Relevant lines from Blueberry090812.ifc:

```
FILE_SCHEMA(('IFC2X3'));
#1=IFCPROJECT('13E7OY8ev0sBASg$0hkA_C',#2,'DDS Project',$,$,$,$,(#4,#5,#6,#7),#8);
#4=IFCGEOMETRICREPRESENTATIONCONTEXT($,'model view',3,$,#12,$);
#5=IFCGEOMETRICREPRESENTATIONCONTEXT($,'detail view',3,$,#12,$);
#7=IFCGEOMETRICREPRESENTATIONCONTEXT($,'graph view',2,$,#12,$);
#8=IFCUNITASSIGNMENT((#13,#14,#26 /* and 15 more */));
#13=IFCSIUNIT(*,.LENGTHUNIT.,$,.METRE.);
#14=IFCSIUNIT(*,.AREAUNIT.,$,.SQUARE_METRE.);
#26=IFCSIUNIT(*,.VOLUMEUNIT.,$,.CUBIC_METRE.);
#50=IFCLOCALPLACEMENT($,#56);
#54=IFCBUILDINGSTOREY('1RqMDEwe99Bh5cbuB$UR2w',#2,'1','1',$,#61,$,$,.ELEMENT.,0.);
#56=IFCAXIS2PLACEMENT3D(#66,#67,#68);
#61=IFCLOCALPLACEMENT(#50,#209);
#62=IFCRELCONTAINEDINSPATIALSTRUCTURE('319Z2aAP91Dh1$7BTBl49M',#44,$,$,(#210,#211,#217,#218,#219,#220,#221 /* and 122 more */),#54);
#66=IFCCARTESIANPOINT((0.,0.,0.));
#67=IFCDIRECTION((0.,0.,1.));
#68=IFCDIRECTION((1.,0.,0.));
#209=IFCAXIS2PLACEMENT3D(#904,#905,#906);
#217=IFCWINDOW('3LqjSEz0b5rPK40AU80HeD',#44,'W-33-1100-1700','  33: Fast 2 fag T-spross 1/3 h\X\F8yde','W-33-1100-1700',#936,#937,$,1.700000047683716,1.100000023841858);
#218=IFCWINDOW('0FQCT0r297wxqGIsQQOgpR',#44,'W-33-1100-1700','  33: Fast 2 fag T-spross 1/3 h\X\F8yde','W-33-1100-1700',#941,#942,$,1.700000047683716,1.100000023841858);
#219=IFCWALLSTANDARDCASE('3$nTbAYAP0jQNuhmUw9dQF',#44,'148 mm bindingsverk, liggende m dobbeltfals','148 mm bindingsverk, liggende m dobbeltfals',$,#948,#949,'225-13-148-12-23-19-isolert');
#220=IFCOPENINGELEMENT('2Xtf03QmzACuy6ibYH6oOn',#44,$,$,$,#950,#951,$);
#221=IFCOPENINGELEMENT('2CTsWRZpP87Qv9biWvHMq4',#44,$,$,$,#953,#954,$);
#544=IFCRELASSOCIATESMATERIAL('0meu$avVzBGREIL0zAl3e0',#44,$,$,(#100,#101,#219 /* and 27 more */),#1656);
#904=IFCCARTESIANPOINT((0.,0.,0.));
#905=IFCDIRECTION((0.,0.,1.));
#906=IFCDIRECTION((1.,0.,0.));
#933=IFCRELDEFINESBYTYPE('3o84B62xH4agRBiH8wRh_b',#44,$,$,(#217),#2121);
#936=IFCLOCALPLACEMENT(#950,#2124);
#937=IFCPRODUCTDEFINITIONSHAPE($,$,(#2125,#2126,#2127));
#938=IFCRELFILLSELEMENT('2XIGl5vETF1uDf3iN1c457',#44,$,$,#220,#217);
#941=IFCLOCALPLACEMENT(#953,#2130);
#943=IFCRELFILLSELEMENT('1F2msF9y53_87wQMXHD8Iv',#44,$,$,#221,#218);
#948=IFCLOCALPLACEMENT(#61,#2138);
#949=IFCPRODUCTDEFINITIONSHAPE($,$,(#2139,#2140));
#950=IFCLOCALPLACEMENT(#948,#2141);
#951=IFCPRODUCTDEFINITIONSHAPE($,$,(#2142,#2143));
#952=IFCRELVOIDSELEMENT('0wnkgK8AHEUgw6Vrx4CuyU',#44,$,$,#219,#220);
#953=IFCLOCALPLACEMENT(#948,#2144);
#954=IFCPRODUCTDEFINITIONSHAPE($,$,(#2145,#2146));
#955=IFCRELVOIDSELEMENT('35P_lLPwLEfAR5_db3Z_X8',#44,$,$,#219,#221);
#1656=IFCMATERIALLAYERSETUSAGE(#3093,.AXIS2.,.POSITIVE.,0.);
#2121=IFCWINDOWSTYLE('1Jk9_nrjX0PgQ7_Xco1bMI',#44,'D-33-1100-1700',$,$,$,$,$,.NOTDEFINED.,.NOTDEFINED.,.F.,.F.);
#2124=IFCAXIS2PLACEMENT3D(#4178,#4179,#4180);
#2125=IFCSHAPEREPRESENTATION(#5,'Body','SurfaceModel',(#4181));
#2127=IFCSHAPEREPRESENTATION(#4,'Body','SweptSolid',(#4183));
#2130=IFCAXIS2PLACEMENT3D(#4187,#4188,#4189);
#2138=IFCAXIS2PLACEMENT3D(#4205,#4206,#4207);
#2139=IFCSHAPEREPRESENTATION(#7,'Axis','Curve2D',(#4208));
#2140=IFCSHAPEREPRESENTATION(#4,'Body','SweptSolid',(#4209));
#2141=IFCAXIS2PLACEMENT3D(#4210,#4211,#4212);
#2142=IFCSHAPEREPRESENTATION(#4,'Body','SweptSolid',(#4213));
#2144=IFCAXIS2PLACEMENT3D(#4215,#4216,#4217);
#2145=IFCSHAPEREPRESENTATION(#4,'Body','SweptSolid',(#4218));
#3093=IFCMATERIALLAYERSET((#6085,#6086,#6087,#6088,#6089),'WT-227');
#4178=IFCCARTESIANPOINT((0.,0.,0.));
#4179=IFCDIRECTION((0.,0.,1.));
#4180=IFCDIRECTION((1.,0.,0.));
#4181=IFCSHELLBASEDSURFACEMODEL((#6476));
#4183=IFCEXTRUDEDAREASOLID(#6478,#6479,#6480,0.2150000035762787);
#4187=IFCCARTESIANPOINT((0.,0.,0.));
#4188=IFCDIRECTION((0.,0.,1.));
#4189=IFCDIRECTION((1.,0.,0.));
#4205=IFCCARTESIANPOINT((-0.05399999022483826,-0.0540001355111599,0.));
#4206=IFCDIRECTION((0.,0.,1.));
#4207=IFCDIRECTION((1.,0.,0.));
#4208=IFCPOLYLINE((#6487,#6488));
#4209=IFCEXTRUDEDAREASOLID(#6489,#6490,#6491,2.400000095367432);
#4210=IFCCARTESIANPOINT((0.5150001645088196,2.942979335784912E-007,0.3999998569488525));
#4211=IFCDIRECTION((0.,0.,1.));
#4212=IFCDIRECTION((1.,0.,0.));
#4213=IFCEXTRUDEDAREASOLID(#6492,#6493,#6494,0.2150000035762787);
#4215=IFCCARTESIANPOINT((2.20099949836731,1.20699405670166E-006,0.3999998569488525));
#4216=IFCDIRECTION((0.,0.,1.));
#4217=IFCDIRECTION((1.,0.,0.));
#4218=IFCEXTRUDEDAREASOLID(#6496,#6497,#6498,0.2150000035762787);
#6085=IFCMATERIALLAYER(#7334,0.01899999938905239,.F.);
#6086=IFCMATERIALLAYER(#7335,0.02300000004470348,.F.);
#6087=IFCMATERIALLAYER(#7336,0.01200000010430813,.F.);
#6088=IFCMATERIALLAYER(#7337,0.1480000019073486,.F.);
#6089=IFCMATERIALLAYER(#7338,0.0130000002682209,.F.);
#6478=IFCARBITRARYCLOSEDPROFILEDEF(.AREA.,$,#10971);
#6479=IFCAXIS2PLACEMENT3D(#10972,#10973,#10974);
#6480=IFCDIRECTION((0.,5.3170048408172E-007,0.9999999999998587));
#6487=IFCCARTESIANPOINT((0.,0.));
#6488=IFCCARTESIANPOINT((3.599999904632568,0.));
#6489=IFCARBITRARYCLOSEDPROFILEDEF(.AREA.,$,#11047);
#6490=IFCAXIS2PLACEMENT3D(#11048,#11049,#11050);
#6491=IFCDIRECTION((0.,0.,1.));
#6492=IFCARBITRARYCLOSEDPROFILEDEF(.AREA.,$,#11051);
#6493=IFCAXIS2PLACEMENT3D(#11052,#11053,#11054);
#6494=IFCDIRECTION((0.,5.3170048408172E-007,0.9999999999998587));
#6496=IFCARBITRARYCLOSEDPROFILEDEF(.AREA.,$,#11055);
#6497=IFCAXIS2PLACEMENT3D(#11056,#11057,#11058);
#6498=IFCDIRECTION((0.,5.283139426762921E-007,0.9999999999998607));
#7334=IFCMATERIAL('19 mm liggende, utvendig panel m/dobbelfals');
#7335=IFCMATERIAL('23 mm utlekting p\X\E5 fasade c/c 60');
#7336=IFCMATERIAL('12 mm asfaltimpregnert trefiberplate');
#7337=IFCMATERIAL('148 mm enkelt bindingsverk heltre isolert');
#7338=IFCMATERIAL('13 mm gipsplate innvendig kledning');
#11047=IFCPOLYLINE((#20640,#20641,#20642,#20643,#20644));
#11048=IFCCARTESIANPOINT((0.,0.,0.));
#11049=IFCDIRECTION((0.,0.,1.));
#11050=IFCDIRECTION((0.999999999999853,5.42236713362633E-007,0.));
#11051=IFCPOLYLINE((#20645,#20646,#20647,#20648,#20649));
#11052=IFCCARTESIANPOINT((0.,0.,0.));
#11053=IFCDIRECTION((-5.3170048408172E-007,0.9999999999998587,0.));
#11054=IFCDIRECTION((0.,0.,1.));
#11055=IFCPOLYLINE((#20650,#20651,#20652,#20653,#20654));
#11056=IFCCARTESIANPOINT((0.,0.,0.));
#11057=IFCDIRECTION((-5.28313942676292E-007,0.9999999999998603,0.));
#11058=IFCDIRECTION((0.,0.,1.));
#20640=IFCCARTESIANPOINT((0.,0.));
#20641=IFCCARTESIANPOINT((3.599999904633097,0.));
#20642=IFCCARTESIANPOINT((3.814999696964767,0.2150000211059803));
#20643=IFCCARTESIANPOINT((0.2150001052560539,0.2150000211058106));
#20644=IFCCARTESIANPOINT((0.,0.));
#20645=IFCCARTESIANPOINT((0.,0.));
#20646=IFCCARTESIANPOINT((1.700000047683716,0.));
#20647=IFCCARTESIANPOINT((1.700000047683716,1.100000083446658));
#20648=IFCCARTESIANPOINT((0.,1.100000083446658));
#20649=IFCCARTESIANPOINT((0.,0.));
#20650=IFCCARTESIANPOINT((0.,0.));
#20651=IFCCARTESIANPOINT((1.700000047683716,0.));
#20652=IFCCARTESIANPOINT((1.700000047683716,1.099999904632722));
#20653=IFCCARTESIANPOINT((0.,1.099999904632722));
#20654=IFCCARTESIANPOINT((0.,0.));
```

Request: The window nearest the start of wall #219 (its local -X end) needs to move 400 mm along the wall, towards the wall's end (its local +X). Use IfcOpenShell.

```python
import ifcopenshell
import ifcopenshell.api.geometry
import ifcopenshell.util.placement
import ifcopenshell.util.unit

model = ifcopenshell.open("Blueberry090812.ifc")
unit_scale = ifcopenshell.util.unit.calculate_unit_scale(model)

window = model.by_guid("3LqjSEz0b5rPK40AU80HeD")
opening = window.FillsVoids[0].RelatingOpeningElement
wall = opening.VoidsElements[0].RelatingBuildingElement

wall_matrix = ifcopenshell.util.placement.get_local_placement(wall.ObjectPlacement)
shift = wall_matrix[:3, 0] * 0.4 / unit_scale
before = ifcopenshell.util.placement.get_local_placement(window.ObjectPlacement)[:3, 3].copy()

# The window is placed relative to its opening, so it follows when the opening moves.
matrix = ifcopenshell.util.placement.get_local_placement(opening.ObjectPlacement)
matrix[:3, 3] += shift
ifcopenshell.api.geometry.edit_object_placement(
    model, product=opening, matrix=matrix, is_si=False, should_transform_children=True
)

after = ifcopenshell.util.placement.get_local_placement(window.ObjectPlacement)[:3, 3]
print("window moved by", (after - before).round(3) + 0.0)

model.write("Blueberry090812_edited.ifc")
```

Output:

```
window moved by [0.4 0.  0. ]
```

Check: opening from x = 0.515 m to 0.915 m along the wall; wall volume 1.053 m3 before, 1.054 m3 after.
